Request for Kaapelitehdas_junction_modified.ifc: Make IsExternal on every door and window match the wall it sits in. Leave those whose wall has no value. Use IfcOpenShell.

First a look at what the model holds.

```python
import ifcopenshell
import ifcopenshell.util.element

model = ifcopenshell.open("Kaapelitehdas_junction_modified.ifc")
print(model.schema)
seen = {}
for e in model.by_type("IfcDoor") + model.by_type("IfcWindow"):
    if not e.FillsVoids:
        continue
    host = e.FillsVoids[0].RelatingOpeningElement.VoidsElements[0].RelatingBuildingElement
    own = ifcopenshell.util.element.get_pset(e, f"Pset_{e.is_a()[3:].removesuffix('StandardCase')}Common", "IsExternal")
    wall = ifcopenshell.util.element.get_pset(host, "Pset_WallCommon", "IsExternal")
    seen[e.is_a(), own, wall] = seen.get((e.is_a(), own, wall), 0) + 1
for (cls, own, wall), count in sorted(seen.items(), key=str):
    print(count, cls, "IsExternal:", own, "| host wall:", wall)
```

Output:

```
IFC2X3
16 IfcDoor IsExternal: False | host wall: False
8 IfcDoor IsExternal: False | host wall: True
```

```python
import ifcopenshell
import ifcopenshell.api.pset
import ifcopenshell.util.element

model = ifcopenshell.open("Kaapelitehdas_junction_modified.ifc")

count = 0
for ifc_class, pset_name in (("IfcDoor", "Pset_DoorCommon"), ("IfcWindow", "Pset_WindowCommon")):
    for e in model.by_type(ifc_class):
        if not e.FillsVoids:
            continue
        host = e.FillsVoids[0].RelatingOpeningElement.VoidsElements[0].RelatingBuildingElement
        external = ifcopenshell.util.element.get_pset(host, "Pset_WallCommon", "IsExternal")
        if external is None or ifcopenshell.util.element.get_pset(e, pset_name, "IsExternal") == external:
            continue
        pset = ifcopenshell.api.pset.add_pset(model, product=e, name=pset_name)
        ifcopenshell.api.pset.edit_pset(model, pset=pset, properties={"IsExternal": external})
        count += 1

print(count, "updated")

model.write("Kaapelitehdas_junction_modified-out.ifc")
```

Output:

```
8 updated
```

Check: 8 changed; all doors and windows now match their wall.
